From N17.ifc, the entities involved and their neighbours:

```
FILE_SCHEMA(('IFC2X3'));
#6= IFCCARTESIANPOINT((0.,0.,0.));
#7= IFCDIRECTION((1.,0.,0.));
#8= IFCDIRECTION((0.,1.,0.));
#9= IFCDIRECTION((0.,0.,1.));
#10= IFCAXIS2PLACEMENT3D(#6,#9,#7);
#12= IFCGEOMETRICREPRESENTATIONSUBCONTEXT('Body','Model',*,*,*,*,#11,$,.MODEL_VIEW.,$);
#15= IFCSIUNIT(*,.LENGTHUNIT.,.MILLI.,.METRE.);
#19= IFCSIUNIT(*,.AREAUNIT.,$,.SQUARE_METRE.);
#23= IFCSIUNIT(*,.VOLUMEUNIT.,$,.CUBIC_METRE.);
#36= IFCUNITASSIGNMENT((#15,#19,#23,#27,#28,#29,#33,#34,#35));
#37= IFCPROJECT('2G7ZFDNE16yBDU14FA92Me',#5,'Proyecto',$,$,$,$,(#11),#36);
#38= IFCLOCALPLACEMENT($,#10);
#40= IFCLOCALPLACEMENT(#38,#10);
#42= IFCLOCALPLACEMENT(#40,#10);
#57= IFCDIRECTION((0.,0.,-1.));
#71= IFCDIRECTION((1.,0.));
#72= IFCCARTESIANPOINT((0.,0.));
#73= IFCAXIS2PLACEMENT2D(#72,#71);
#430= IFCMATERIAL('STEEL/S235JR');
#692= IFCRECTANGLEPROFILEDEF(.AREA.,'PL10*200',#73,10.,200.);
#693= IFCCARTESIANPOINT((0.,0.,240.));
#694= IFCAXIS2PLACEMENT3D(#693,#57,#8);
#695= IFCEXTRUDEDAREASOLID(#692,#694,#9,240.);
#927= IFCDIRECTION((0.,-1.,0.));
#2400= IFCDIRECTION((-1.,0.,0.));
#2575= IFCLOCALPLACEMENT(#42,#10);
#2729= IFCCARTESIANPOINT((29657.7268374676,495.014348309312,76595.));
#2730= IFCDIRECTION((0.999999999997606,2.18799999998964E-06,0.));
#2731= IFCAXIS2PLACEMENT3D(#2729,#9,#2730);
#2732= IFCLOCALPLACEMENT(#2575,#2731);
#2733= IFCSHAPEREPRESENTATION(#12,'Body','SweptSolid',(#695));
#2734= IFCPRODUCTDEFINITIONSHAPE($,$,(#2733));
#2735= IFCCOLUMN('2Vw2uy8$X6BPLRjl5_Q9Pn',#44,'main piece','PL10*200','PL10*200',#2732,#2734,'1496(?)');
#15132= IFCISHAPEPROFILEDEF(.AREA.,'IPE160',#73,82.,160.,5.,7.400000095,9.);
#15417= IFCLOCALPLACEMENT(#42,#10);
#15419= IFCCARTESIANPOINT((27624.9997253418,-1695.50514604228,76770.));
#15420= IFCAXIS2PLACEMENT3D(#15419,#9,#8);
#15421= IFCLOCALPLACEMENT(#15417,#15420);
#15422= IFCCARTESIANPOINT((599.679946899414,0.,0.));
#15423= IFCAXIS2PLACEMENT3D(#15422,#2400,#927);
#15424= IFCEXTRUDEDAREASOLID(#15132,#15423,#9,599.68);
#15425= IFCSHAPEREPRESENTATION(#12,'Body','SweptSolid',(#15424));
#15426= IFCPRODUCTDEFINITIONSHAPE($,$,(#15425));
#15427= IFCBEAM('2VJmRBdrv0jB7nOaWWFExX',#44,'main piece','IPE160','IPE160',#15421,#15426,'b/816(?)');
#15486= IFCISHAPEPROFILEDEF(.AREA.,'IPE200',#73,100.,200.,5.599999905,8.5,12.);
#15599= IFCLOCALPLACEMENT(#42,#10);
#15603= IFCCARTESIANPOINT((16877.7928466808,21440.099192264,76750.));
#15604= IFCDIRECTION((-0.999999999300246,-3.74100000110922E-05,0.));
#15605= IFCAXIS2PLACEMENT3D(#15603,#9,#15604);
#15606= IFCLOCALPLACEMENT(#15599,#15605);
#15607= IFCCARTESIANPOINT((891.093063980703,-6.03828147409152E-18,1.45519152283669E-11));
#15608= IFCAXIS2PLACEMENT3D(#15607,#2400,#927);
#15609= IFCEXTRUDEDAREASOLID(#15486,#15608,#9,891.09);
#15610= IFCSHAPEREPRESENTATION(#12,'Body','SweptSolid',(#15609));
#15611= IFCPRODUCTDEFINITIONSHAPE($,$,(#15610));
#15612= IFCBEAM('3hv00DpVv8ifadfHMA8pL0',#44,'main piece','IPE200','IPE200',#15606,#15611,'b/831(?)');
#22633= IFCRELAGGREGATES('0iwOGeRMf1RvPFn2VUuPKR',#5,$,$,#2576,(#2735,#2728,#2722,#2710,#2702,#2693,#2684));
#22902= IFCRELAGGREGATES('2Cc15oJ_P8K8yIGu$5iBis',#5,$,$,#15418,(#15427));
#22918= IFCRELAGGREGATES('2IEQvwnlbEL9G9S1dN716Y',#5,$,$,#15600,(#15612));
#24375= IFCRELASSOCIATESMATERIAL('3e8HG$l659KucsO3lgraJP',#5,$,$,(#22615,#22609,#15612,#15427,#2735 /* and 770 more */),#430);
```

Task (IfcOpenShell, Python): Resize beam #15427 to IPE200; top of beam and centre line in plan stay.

```python
import ifcopenshell
import ifcopenshell.util.element
import ifcopenshell.util.representation

model = ifcopenshell.open("N17.ifc")

member = model.by_guid("2VJmRBdrv0jB7nOaWWFExX")
source = next(p for p in model.by_type("IfcIShapeProfileDef") if p.ProfileName == "IPE200")

body = ifcopenshell.util.representation.get_representation(member, "Model", "Body")
solid = body.Items[0]
old_profile = solid.SweptArea

# Copy the section's sizes but keep this member's own profile position.
profile = ifcopenshell.util.element.copy(model, source)
# Profiles are centred, so shift by half the change in depth to hold the top.
shift = (old_profile.OverallDepth - profile.OverallDepth) / 2
x, y = old_profile.Position.Location.Coordinates
up = (0.0, 1.0)  # upwards, in the solid's own plane
location = model.createIfcCartesianPoint((x + up[0] * shift, y + up[1] * shift))
profile.Position = model.createIfcAxis2Placement2D(location, old_profile.Position.RefDirection)
solid.SweptArea = profile
if not model.get_total_inverses(old_profile):
    ifcopenshell.util.element.remove_deep2(model, old_profile)
member.Description = member.Description.replace("IPE160", "IPE200")
member.ObjectType = member.ObjectType.replace("IPE160", "IPE200")

print(solid.SweptArea)

model.write("N17_v2.ifc")
```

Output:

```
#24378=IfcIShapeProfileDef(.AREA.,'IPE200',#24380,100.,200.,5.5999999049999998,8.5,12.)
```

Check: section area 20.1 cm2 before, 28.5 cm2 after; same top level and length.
